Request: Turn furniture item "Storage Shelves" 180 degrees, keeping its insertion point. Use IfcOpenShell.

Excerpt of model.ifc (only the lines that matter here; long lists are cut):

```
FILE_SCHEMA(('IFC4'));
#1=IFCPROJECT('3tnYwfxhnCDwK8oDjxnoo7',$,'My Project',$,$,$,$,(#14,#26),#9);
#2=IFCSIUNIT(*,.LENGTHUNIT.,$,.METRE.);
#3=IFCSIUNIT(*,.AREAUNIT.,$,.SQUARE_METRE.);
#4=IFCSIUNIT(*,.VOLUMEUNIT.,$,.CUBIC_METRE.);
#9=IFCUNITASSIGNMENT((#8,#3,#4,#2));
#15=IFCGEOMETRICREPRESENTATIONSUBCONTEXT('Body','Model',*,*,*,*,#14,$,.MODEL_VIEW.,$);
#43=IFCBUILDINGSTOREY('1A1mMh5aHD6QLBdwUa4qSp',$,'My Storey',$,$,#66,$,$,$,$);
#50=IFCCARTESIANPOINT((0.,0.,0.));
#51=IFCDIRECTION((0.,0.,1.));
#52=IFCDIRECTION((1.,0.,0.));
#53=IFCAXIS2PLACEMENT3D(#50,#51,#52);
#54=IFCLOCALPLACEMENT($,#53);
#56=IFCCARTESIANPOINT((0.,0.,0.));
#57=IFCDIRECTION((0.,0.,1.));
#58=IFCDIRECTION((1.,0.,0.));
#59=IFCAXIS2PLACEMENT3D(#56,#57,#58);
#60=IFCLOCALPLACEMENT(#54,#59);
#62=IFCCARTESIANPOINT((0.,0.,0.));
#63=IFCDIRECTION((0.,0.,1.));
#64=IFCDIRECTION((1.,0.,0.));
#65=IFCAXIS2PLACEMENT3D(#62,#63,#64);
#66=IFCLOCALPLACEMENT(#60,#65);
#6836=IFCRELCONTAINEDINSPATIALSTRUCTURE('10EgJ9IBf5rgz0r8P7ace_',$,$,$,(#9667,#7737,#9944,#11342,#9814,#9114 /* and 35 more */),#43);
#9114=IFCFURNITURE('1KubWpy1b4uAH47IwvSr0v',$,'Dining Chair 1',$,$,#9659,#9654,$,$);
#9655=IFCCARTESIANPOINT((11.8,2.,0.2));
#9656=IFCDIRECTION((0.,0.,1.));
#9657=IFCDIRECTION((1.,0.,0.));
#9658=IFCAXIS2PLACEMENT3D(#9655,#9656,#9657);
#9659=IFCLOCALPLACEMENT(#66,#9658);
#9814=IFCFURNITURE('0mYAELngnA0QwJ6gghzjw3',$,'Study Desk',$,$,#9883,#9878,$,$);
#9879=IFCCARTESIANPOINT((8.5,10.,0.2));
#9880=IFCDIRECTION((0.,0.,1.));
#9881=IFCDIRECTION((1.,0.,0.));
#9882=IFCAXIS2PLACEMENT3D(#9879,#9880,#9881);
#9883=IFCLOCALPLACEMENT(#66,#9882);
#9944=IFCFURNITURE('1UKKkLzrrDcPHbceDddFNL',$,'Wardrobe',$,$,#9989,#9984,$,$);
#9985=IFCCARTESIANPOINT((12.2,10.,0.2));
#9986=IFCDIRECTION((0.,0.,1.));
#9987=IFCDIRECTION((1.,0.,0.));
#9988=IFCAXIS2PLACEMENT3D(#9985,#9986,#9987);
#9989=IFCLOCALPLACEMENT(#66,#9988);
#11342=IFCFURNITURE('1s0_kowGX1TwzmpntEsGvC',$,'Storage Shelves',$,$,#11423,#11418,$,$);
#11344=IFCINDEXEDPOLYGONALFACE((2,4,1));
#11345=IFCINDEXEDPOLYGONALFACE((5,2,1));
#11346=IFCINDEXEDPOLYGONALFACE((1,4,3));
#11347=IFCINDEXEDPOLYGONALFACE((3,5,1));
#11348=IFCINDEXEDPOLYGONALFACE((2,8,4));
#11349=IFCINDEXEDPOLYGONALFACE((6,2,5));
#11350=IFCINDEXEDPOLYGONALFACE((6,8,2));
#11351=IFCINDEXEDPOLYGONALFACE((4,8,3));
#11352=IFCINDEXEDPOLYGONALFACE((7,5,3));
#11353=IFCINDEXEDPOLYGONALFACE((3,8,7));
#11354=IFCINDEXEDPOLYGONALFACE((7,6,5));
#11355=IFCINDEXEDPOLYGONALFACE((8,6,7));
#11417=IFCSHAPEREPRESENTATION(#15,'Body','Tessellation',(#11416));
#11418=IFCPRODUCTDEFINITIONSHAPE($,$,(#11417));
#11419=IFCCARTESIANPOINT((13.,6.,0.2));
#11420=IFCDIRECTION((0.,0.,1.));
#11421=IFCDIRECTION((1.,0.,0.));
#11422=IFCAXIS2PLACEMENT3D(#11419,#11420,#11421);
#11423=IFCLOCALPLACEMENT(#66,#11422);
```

```python
import ifcopenshell
import ifcopenshell.api.geometry
import ifcopenshell.util.placement

model = ifcopenshell.open("model.ifc")

item = model.by_id(11342)
matrix = ifcopenshell.util.placement.get_local_placement(item.ObjectPlacement)
matrix = matrix @ ifcopenshell.util.placement.rotation(180, "Z")
ifcopenshell.api.geometry.edit_object_placement(model, product=item, matrix=matrix, is_si=False)

print(ifcopenshell.util.placement.get_local_placement(item.ObjectPlacement).round(3) + 0.0)

model.write("model_updated.ifc")
```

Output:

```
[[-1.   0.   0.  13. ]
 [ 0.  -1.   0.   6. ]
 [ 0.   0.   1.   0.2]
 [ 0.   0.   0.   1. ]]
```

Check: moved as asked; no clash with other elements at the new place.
